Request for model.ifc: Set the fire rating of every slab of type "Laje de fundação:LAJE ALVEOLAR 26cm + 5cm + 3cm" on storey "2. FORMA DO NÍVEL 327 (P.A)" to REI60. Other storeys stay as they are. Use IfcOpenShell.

First a look at what the model holds.

```python
import ifcopenshell
import ifcopenshell.util.element

model = ifcopenshell.open("model.ifc")
print(model.schema)
storey = next(s for s in model.by_type("IfcBuildingStorey") if s.Name == "2. FORMA DO NÍVEL 327 (P.A)")
slabs = [e for e in ifcopenshell.util.element.get_decomposition(storey) if e.is_a("IfcSlab")]
seen = {}
for e in slabs:
    element_type = ifcopenshell.util.element.get_type(e)
    key = (element_type.Name if element_type != e and element_type else None, ifcopenshell.util.element.get_pset(e, "Pset_SlabCommon", "FireRating"))
    seen[key] = seen.get(key, 0) + 1
for (name, value), count in sorted(seen.items(), key=str):
    print(count, "x", name, "|", value)
```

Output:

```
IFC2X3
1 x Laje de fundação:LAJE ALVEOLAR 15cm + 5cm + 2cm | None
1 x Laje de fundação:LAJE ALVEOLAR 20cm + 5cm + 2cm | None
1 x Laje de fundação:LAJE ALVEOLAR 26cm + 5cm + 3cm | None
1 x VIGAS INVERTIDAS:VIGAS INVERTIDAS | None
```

```python
import ifcopenshell
import ifcopenshell.api.pset
import ifcopenshell.util.element

model = ifcopenshell.open("model.ifc")

storey = next(s for s in model.by_type("IfcBuildingStorey") if s.Name == "2. FORMA DO NÍVEL 327 (P.A)")
slabs = [e for e in ifcopenshell.util.element.get_decomposition(storey) if e.is_a("IfcSlab")]

count = 0
for e in slabs:
    element_type = ifcopenshell.util.element.get_type(e)
    if element_type in (None, e) or element_type.Name != "Laje de fundação:LAJE ALVEOLAR 26cm + 5cm + 3cm":
        continue
    # add_pset returns the element's existing set when there is one.
    pset = ifcopenshell.api.pset.add_pset(model, product=e, name="Pset_SlabCommon")
    ifcopenshell.api.pset.edit_pset(model, pset=pset, properties={"FireRating": "REI60"})
    count += 1

print(count, "slabs updated")

model.write("model_edited.ifc")
```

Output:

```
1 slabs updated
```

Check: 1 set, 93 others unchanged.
